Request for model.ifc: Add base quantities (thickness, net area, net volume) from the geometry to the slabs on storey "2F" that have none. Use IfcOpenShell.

First a look at what the model holds.

```python
import ifcopenshell
import ifcopenshell.util.element
import ifcopenshell.util.unit

model = ifcopenshell.open("model.ifc")
print(model.schema)
for unit_type in ("LENGTHUNIT", "AREAUNIT", "VOLUMEUNIT"):
    print(unit_type, ifcopenshell.util.unit.calculate_unit_scale(model, unit_type))
storey = next(s for s in model.by_type("IfcBuildingStorey") if s.Name == "2F")
slabs = [e for e in ifcopenshell.util.element.get_decomposition(storey) if e.is_a("IfcSlab")]
for e in sorted(slabs, key=lambda e: e.id()):
    print(e.id(), e.is_a(), e.Name, list(ifcopenshell.util.element.get_psets(e, qtos_only=True)), sep=" | ")
```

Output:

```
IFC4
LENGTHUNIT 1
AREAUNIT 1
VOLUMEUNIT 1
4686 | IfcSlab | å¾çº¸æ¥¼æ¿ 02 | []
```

```python
import ifcopenshell
import ifcopenshell.api.pset
import ifcopenshell.geom
import ifcopenshell.util.element
import ifcopenshell.util.shape
import ifcopenshell.util.unit

model = ifcopenshell.open("model.ifc")
unit_scale = ifcopenshell.util.unit.calculate_unit_scale(model)
area_scale = ifcopenshell.util.unit.calculate_unit_scale(model, "AREAUNIT")
volume_scale = ifcopenshell.util.unit.calculate_unit_scale(model, "VOLUMEUNIT")
settings = ifcopenshell.geom.settings()

storey = next(s for s in model.by_type("IfcBuildingStorey") if s.Name == "2F")
slabs = [e for e in ifcopenshell.util.element.get_decomposition(storey) if e.is_a("IfcSlab")]

for e in sorted(slabs, key=lambda e: e.id()):
    if ifcopenshell.util.element.get_psets(e, qtos_only=True, should_inherit=False):
        continue
    # Geometry comes back in metres, in the element's own axes.
    shape = ifcopenshell.geom.create_shape(settings, e)
    values = {
        "Width": ifcopenshell.util.shape.get_z(shape.geometry) / unit_scale,
        "NetArea": ifcopenshell.util.shape.get_footprint_area(shape.geometry) / area_scale,
        "NetVolume": ifcopenshell.util.shape.get_volume(shape.geometry) / volume_scale,
    }
    qto = ifcopenshell.api.pset.add_qto(model, product=e, name="Qto_SlabBaseQuantities")
    ifcopenshell.api.pset.edit_qto(model, qto=qto, properties=values)
    print(e.id(), {k: round(v, 3) for k, v in values.items()})

model.write("model_updated.ifc")
```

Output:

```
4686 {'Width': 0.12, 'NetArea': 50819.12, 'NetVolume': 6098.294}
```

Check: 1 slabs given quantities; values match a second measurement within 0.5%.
